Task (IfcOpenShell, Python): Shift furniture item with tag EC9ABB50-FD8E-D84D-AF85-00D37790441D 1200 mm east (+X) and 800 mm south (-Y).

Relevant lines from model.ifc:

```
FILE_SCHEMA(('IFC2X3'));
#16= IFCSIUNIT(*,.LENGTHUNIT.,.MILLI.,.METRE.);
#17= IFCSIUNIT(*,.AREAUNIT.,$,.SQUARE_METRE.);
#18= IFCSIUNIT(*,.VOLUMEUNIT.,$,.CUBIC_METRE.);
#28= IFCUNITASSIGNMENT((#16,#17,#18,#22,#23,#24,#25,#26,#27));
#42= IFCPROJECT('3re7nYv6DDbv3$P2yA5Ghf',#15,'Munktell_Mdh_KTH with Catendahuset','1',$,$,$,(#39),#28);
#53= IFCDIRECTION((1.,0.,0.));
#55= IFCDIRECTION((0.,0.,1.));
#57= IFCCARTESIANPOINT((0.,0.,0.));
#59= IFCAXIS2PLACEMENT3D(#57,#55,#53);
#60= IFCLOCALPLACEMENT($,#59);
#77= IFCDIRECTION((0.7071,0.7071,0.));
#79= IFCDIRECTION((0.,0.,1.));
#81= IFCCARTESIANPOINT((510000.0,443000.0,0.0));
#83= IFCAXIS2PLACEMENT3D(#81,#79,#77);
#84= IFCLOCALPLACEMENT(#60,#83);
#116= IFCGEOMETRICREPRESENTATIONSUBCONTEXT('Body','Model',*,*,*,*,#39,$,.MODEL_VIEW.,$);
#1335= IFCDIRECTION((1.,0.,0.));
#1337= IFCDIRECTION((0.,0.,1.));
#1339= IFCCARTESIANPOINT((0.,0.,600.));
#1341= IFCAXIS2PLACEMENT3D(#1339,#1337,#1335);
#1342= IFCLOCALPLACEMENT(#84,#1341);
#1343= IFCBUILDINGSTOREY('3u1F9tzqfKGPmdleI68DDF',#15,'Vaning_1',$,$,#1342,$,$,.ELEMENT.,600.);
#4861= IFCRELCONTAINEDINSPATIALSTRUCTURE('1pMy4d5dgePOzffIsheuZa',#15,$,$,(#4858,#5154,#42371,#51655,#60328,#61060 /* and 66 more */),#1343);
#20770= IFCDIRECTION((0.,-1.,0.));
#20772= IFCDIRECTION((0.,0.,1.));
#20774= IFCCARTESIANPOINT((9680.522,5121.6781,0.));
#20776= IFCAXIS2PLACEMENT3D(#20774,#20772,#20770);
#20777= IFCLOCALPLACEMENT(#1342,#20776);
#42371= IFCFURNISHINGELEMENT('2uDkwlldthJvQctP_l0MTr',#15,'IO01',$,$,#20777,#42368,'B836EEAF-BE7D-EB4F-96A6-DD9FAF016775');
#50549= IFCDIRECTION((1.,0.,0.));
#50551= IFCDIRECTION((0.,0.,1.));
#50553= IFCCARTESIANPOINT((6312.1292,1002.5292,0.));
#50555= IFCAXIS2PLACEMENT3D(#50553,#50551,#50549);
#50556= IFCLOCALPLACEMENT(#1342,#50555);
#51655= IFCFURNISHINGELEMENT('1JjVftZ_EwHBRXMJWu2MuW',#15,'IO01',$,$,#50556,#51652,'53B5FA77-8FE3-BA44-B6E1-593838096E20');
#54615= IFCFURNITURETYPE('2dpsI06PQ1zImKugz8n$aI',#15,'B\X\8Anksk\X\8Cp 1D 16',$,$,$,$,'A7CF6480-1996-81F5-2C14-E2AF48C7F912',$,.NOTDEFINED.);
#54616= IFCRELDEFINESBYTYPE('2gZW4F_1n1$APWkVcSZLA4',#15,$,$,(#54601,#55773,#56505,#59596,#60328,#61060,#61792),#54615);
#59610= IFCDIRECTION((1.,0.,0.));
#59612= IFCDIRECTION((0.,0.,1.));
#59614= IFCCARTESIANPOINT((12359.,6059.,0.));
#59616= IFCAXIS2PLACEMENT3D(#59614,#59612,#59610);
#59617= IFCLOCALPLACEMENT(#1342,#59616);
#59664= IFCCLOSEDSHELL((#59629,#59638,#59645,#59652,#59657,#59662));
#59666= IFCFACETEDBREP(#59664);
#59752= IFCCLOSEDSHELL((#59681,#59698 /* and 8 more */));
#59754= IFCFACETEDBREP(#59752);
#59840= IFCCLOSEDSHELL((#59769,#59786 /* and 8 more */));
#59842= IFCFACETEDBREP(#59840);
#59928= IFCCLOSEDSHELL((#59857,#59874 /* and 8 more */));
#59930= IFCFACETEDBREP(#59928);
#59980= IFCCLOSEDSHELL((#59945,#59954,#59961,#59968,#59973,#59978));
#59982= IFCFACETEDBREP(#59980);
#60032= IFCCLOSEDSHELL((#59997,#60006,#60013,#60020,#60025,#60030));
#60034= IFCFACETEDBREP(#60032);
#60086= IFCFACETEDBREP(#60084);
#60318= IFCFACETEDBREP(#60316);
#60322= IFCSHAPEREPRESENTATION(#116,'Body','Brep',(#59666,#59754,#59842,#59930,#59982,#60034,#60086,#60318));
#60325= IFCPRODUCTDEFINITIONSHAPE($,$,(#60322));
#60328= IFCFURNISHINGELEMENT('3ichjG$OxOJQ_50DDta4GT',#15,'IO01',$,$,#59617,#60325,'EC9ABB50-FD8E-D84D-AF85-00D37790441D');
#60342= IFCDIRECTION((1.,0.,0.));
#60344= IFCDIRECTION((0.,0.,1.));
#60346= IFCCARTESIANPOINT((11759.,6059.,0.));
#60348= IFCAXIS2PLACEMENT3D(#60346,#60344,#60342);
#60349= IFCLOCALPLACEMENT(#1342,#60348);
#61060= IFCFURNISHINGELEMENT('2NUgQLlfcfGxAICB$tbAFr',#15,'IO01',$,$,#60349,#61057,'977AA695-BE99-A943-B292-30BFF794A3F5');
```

```python
import ifcopenshell
import ifcopenshell.api.geometry
import ifcopenshell.util.placement
import ifcopenshell.util.unit

model = ifcopenshell.open("model.ifc")
unit_scale = ifcopenshell.util.unit.calculate_unit_scale(model)

item = model.by_guid("3ichjG$OxOJQ_50DDta4GT")
matrix = ifcopenshell.util.placement.get_local_placement(item.ObjectPlacement)
matrix[0, 3] += 1.2 / unit_scale
matrix[1, 3] -= 0.8 / unit_scale
ifcopenshell.api.geometry.edit_object_placement(model, product=item, matrix=matrix, is_si=False)

print(ifcopenshell.util.placement.get_local_placement(item.ObjectPlacement).round(3) + 0.0)

model.write("model_updated.ifc")
```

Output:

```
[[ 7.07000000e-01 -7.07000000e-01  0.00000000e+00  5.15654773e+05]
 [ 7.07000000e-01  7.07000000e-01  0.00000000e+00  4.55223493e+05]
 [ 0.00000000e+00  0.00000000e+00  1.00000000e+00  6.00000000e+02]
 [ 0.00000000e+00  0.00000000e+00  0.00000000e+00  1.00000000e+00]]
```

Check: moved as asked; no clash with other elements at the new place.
